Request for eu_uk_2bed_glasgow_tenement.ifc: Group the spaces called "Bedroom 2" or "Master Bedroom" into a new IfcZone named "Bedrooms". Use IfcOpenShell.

First a look at what the model holds.

```python
import ifcopenshell

model = ifcopenshell.open("eu_uk_2bed_glasgow_tenement.ifc")
print(model.schema)
seen = {}
for space in model.by_type("IfcSpace"):
    seen[space.LongName] = seen.get(space.LongName, 0) + 1
for name, count in sorted(seen.items(), key=str):
    print(count, "x", name)
print("zones:", [z.Name for z in model.by_type("IfcZone")][:20])
```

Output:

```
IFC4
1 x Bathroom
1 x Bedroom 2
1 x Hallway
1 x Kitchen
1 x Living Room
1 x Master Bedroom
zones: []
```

```python
import ifcopenshell
import ifcopenshell.api.group
import ifcopenshell.api.root

model = ifcopenshell.open("eu_uk_2bed_glasgow_tenement.ifc")

names = {"Bedroom 2", "Master Bedroom"}
spaces = [s for s in model.by_type("IfcSpace") if s.LongName in names]

zone = ifcopenshell.api.root.create_entity(model, ifc_class="IfcZone", name="Bedrooms")
ifcopenshell.api.group.assign_group(model, products=spaces, group=zone)
print(len(spaces), "spaces in", zone.Name)

model.write("eu_uk_2bed_glasgow_tenement_rev.ifc")
```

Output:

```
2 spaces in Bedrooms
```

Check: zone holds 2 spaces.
